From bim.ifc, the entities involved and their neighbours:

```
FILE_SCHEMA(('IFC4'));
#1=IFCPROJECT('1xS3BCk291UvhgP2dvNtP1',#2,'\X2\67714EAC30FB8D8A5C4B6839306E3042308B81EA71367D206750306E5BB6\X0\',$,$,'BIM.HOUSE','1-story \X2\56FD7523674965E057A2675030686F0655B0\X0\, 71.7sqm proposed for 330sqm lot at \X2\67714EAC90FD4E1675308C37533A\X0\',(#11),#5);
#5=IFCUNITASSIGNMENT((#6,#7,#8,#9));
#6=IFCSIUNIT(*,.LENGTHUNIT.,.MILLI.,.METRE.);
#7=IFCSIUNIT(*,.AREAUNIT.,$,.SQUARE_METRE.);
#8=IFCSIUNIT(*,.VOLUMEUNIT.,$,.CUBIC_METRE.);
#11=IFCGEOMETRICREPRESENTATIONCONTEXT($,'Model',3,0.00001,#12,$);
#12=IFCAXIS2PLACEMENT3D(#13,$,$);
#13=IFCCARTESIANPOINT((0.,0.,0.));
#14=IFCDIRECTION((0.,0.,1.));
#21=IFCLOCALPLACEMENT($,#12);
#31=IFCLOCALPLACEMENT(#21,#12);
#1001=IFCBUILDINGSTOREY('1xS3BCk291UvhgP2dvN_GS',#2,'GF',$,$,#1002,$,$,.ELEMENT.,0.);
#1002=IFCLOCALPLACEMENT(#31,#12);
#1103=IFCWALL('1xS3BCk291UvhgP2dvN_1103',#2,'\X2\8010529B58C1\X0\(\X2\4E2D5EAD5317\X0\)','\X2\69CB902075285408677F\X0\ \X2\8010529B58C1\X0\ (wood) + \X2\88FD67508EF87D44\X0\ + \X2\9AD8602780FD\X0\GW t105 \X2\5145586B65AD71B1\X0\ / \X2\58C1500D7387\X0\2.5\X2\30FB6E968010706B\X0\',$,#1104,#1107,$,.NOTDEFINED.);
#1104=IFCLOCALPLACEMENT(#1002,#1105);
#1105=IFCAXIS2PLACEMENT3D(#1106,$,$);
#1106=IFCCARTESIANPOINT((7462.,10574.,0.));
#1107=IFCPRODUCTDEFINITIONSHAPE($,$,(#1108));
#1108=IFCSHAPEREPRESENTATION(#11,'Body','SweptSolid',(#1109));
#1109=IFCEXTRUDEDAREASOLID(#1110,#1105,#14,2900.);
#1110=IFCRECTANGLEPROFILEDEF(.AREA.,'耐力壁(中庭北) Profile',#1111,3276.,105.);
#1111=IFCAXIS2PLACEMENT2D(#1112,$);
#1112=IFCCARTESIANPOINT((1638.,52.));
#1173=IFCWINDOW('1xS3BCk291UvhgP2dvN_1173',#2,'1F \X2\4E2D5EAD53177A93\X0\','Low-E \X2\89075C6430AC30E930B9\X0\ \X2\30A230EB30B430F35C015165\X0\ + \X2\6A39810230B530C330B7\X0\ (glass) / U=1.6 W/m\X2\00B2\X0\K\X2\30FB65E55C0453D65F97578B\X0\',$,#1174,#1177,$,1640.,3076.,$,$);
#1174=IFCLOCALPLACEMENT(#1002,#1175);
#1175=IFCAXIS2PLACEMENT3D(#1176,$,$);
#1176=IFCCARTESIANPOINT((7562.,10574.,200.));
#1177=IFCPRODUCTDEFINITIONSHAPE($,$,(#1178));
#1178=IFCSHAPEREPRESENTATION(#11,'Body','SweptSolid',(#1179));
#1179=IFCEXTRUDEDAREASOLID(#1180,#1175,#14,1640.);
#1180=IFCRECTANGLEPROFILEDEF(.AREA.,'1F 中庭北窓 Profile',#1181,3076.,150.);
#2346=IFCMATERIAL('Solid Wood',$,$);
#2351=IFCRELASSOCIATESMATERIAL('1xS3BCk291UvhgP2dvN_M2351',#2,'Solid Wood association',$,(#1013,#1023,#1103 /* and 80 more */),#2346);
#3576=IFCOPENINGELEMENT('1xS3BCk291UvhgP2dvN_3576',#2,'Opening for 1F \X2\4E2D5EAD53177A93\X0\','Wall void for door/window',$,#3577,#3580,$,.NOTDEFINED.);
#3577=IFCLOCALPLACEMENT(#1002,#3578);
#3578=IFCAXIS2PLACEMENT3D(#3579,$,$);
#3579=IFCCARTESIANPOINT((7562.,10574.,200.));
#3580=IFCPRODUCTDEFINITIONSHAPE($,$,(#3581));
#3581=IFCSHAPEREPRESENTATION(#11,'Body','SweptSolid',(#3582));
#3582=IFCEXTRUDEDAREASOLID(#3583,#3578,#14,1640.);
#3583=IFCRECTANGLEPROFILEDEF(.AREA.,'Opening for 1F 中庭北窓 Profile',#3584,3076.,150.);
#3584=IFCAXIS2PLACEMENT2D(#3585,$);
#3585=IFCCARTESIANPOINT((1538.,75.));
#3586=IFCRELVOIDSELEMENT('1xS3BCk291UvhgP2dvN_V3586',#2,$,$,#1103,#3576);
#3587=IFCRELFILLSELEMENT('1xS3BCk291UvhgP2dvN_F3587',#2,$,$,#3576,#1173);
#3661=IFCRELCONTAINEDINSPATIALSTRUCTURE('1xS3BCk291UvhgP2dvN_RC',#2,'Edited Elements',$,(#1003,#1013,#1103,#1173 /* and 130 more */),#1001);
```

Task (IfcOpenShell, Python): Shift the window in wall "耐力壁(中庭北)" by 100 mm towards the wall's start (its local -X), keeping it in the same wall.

```python
import ifcopenshell
import ifcopenshell.api.geometry
import ifcopenshell.util.placement
import ifcopenshell.util.unit

model = ifcopenshell.open("bim.ifc")
unit_scale = ifcopenshell.util.unit.calculate_unit_scale(model)

window = model.by_id(1173)
opening = window.FillsVoids[0].RelatingOpeningElement
wall = opening.VoidsElements[0].RelatingBuildingElement

wall_matrix = ifcopenshell.util.placement.get_local_placement(wall.ObjectPlacement)
shift = wall_matrix[:3, 0] * -0.1 / unit_scale
before = ifcopenshell.util.placement.get_local_placement(window.ObjectPlacement)[:3, 3].copy()

# The window is not placed relative to its opening, so move both.
for product in (opening, window):
    matrix = ifcopenshell.util.placement.get_local_placement(product.ObjectPlacement)
    matrix[:3, 3] += shift
    ifcopenshell.api.geometry.edit_object_placement(model, product=product, matrix=matrix, is_si=False)

after = ifcopenshell.util.placement.get_local_placement(window.ObjectPlacement)[:3, 3]
print("window moved by", (after - before).round(3) + 0.0)

model.write("bim_rev.ifc")
```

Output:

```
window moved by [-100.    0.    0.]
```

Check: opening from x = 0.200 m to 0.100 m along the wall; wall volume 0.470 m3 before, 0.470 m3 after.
